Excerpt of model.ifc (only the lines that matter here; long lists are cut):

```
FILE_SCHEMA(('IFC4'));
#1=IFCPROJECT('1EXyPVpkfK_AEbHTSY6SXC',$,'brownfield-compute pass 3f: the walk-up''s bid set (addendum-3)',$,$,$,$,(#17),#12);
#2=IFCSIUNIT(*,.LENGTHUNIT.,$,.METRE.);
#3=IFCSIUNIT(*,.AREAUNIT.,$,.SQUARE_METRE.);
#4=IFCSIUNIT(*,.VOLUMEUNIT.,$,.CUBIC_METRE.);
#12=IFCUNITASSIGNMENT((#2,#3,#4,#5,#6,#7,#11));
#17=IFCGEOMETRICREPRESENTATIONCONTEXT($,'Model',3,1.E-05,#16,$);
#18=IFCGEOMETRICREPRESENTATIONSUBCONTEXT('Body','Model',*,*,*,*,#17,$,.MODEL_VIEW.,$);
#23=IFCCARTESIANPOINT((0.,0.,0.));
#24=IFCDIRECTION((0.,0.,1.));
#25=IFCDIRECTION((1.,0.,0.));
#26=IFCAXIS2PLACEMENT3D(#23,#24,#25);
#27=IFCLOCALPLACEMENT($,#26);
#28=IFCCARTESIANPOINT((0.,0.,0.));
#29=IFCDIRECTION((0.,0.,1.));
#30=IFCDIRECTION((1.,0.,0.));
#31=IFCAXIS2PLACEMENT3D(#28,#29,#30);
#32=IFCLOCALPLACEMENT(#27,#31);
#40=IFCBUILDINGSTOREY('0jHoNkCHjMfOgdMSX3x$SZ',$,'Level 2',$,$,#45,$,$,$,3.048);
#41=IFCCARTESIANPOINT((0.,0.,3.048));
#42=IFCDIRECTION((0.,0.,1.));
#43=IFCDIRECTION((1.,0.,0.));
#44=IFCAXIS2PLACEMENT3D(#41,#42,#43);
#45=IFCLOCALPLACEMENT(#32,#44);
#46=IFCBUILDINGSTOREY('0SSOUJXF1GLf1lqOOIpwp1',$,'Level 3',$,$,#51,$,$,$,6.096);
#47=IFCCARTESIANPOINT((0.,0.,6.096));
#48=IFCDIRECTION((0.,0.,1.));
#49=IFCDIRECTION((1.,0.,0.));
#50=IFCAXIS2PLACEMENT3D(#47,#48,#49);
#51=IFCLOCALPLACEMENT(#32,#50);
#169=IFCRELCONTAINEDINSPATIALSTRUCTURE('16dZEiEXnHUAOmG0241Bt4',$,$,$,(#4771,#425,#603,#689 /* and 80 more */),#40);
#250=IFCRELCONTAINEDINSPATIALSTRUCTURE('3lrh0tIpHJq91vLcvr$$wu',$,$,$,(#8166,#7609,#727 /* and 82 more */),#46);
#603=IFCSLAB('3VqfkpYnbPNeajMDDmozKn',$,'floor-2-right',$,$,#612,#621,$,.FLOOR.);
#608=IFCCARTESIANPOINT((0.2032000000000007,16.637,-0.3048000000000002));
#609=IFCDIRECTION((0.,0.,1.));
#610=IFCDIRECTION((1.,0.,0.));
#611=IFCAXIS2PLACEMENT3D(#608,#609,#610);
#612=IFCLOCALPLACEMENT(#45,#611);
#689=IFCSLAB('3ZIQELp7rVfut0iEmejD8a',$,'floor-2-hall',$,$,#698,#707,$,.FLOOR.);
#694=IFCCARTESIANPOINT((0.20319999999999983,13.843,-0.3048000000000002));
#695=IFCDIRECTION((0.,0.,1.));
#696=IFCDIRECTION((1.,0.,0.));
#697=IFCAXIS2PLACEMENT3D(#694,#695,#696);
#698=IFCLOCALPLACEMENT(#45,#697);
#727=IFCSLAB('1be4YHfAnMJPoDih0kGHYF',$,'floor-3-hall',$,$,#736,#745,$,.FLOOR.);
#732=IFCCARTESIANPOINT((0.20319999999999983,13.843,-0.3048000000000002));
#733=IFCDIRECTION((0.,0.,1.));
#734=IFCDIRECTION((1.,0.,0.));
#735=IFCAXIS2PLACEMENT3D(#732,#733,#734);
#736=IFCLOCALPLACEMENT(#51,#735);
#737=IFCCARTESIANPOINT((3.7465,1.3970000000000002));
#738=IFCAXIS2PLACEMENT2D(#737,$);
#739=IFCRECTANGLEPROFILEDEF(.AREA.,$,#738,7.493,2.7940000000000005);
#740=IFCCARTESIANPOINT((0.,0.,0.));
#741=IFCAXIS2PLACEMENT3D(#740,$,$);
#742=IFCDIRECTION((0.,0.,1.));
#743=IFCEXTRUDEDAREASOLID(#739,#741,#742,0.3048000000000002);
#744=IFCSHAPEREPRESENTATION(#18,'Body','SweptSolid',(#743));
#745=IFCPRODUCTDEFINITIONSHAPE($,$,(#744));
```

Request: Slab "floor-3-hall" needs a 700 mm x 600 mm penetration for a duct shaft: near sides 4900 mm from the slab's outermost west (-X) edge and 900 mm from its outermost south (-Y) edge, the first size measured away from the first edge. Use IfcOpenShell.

```python
import numpy as np
import ifcopenshell
import ifcopenshell.api.feature
import ifcopenshell.api.geometry
import ifcopenshell.api.root
import ifcopenshell.geom
import ifcopenshell.util.placement
import ifcopenshell.util.representation
import ifcopenshell.util.shape
import ifcopenshell.util.unit

model = ifcopenshell.open("model.ifc")
unit_scale = ifcopenshell.util.unit.calculate_unit_scale(model)
settings = ifcopenshell.geom.settings()


def volume(element):
    """Net volume in cubic metres, openings subtracted."""
    shape = ifcopenshell.geom.create_shape(settings, element)
    return ifcopenshell.util.shape.get_volume(shape.geometry)


slab = model.by_guid("1be4YHfAnMJPoDih0kGHYF")
before = volume(slab)

# Extent in the slab's own axes, in metres. The edges named are its -X and -Y sides.
slab_shape = ifcopenshell.geom.create_shape(settings, slab)
vertices = ifcopenshell.util.shape.get_vertices(slab_shape.geometry)
x_min, y_min, bottom = vertices.min(axis=0)
top = vertices[:, 2].max()

opening = ifcopenshell.api.root.create_entity(model, ifc_class="IfcOpeningElement", name="Duct shaft opening", predefined_type="OPENING")
context = ifcopenshell.util.representation.get_context(model, "Model", "Body", "MODEL_VIEW")
width, depth = 0.7, 0.6
outline = [(0.0, 0.0), (width, 0.0), (width, depth), (0.0, depth), (0.0, 0.0)]
# Overshoot both faces by 50 mm so the cut is clean.
shape = ifcopenshell.api.geometry.add_slab_representation(
    model, context=context, depth=top - bottom + 0.1, polyline=outline
)
ifcopenshell.api.geometry.assign_representation(model, product=opening, representation=shape)

matrix = ifcopenshell.util.placement.get_local_placement(slab.ObjectPlacement)
matrix[:, 3] = matrix @ np.append(np.array([x_min + 4.9, y_min + 0.9, bottom - 0.05]) / unit_scale, 1.0)
ifcopenshell.api.geometry.edit_object_placement(model, product=opening, matrix=matrix, is_si=False)
ifcopenshell.api.feature.add_feature(model, feature=opening, element=slab)

after = volume(slab)

print(f"slab volume {before:.3f} -> {after:.3f} m3")

model.write("model_v2.ifc")
```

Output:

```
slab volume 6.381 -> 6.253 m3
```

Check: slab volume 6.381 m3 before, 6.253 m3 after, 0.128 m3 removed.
